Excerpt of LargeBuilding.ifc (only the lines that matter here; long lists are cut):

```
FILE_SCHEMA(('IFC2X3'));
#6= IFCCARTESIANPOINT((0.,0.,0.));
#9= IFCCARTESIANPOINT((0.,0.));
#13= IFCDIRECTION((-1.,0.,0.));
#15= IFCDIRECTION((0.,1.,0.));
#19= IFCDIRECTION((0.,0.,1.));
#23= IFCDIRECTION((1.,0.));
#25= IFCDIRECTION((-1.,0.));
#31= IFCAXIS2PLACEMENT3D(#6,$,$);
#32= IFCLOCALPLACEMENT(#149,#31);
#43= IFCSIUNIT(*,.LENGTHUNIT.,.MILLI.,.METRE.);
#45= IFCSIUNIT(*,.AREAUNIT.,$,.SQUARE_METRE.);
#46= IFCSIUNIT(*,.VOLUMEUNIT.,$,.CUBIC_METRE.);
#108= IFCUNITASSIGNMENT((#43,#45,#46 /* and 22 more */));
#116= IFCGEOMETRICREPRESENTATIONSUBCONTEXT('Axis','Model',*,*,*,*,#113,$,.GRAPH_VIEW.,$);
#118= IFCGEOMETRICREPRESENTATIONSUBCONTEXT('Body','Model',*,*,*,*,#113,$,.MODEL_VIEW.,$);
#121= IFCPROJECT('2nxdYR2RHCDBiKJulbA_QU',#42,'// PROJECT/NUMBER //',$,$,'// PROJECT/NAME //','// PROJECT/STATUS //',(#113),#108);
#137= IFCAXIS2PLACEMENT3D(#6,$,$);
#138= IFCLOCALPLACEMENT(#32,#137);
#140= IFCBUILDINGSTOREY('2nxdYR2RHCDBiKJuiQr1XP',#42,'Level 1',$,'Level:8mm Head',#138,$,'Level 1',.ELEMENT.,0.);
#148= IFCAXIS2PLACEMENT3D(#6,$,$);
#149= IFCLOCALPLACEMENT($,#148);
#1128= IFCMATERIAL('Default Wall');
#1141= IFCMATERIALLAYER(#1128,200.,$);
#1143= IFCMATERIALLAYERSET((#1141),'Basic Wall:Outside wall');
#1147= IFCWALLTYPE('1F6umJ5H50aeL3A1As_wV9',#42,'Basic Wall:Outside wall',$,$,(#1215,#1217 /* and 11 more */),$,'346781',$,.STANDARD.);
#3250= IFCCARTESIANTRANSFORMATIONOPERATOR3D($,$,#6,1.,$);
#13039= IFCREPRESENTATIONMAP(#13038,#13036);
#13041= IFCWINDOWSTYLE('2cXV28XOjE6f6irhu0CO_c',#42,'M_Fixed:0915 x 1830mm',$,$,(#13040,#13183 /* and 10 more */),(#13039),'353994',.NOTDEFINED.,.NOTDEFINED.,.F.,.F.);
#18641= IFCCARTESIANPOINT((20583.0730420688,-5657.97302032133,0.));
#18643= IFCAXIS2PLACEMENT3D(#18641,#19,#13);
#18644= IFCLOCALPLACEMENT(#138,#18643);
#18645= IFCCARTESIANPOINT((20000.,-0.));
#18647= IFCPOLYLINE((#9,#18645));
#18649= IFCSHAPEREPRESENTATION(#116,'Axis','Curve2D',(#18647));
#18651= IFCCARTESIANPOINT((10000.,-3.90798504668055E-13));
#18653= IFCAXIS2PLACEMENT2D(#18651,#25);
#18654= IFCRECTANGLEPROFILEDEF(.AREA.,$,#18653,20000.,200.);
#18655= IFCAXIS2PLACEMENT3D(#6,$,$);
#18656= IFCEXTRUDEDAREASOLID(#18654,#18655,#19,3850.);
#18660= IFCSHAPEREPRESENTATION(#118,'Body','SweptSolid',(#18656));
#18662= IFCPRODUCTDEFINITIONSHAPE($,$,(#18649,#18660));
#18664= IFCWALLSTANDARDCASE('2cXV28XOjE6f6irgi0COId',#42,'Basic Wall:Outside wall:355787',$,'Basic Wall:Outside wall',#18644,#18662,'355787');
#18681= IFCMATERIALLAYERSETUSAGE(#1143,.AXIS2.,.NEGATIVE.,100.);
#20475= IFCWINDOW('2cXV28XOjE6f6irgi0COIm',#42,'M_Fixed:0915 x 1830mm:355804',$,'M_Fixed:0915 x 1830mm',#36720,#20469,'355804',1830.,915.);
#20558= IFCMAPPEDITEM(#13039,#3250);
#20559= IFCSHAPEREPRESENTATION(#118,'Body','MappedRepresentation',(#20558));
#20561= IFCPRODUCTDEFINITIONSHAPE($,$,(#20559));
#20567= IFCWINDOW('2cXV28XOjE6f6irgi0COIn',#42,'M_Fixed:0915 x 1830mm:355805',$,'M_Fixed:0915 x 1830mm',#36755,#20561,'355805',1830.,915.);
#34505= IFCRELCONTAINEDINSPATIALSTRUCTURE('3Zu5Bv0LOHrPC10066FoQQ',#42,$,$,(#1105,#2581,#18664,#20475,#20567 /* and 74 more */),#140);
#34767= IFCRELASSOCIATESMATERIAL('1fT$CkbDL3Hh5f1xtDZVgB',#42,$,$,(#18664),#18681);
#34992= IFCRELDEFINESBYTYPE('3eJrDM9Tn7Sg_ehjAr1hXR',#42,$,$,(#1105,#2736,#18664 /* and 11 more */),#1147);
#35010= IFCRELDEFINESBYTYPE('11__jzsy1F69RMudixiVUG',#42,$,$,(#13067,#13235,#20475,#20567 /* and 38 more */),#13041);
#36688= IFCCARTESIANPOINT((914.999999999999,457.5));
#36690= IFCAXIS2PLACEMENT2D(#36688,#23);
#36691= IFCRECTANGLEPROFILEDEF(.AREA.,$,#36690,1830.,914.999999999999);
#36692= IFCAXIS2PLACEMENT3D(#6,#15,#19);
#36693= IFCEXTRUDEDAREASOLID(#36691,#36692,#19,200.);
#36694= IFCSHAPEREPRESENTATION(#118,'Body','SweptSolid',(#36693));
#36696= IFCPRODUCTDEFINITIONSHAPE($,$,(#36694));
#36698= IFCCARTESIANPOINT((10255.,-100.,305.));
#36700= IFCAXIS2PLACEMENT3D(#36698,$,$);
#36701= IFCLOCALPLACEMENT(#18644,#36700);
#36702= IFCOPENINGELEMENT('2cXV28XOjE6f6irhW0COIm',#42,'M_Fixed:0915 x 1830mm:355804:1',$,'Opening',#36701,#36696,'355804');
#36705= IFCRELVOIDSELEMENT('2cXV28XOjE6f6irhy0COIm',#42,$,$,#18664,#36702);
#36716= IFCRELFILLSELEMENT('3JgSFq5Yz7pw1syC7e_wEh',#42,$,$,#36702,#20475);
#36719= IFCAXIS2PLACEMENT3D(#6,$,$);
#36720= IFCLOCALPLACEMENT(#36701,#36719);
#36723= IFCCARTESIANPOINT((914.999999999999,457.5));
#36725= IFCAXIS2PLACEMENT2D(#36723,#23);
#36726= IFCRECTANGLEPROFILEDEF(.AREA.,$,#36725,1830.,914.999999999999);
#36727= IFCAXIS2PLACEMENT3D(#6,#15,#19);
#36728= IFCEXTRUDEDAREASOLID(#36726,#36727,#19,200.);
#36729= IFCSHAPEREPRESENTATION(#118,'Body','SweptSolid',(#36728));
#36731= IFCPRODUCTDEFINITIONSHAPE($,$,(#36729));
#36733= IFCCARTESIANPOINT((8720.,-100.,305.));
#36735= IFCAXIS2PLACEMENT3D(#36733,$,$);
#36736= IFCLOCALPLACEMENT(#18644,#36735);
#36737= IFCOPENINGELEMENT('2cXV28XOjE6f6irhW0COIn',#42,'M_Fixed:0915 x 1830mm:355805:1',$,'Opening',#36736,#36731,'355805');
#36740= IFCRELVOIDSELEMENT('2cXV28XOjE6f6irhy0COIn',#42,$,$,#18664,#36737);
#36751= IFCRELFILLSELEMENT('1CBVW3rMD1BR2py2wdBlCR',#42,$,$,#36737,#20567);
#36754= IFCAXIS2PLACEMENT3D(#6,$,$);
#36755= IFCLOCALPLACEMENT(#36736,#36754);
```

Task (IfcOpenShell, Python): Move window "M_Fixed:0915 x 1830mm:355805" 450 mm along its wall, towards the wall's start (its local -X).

```python
import ifcopenshell
import ifcopenshell.api.geometry
import ifcopenshell.util.placement

model = ifcopenshell.open("LargeBuilding.ifc")

window = model.by_guid("2cXV28XOjE6f6irgi0COIn")
opening = window.FillsVoids[0].RelatingOpeningElement
wall = opening.VoidsElements[0].RelatingBuildingElement

wall_matrix = ifcopenshell.util.placement.get_local_placement(wall.ObjectPlacement)
shift = wall_matrix[:3, 0] * -450.0
before = ifcopenshell.util.placement.get_local_placement(window.ObjectPlacement)[:3, 3].copy()

# The window is placed relative to its opening, so it follows when the opening moves.
matrix = ifcopenshell.util.placement.get_local_placement(opening.ObjectPlacement)
matrix[:3, 3] += shift
ifcopenshell.api.geometry.edit_object_placement(
    model, product=opening, matrix=matrix, is_si=False, should_transform_children=True
)

after = ifcopenshell.util.placement.get_local_placement(window.ObjectPlacement)[:3, 3]
print("window moved by", (after - before).round(3) + 0.0)

model.write("LargeBuilding_v2.ifc")
```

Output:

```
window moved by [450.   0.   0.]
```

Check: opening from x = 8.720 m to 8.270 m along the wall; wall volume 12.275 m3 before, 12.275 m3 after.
